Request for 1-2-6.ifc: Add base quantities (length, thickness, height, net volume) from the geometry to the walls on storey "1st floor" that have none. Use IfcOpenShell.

First a look at what the model holds.

```python
import ifcopenshell
import ifcopenshell.util.element
import ifcopenshell.util.unit

model = ifcopenshell.open("1-2-6.ifc")
print(model.schema)
for unit_type in ("LENGTHUNIT", "AREAUNIT", "VOLUMEUNIT"):
    print(unit_type, ifcopenshell.util.unit.calculate_unit_scale(model, unit_type))
storey = next(s for s in model.by_type("IfcBuildingStorey") if s.Name == "1st floor")
walls = [e for e in ifcopenshell.util.element.get_decomposition(storey) if e.is_a("IfcWall")]
for e in sorted(walls, key=lambda e: e.id()):
    print(e.id(), e.is_a(), e.Name, list(ifcopenshell.util.element.get_psets(e, qtos_only=True)), sep=" | ")
```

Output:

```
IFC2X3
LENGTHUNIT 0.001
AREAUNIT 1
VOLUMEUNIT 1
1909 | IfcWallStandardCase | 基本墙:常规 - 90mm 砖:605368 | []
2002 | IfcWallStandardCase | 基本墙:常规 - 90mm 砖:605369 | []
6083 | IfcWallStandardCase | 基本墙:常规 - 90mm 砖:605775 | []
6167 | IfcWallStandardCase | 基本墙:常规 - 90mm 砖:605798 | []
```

```python
import ifcopenshell
import ifcopenshell.api.pset
import ifcopenshell.geom
import ifcopenshell.util.element
import ifcopenshell.util.shape
import ifcopenshell.util.unit

model = ifcopenshell.open("1-2-6.ifc")
unit_scale = ifcopenshell.util.unit.calculate_unit_scale(model)
volume_scale = ifcopenshell.util.unit.calculate_unit_scale(model, "VOLUMEUNIT")
settings = ifcopenshell.geom.settings()

storey = next(s for s in model.by_type("IfcBuildingStorey") if s.Name == "1st floor")
walls = [e for e in ifcopenshell.util.element.get_decomposition(storey) if e.is_a("IfcWall")]

for e in sorted(walls, key=lambda e: e.id()):
    if ifcopenshell.util.element.get_psets(e, qtos_only=True, should_inherit=False):
        continue
    # Geometry comes back in metres, in the element's own axes.
    shape = ifcopenshell.geom.create_shape(settings, e)
    values = {
        "Length": ifcopenshell.util.shape.get_x(shape.geometry) / unit_scale,
        "Width": ifcopenshell.util.shape.get_y(shape.geometry) / unit_scale,
        "Height": ifcopenshell.util.shape.get_z(shape.geometry) / unit_scale,
        "NetVolume": ifcopenshell.util.shape.get_volume(shape.geometry) / volume_scale,
    }
    qto = ifcopenshell.api.pset.add_qto(model, product=e, name="BaseQuantities")
    ifcopenshell.api.pset.edit_qto(model, qto=qto, properties=values)
    print(e.id(), {k: round(v, 3) for k, v in values.items()})

model.write("1-2-6_updated.ifc")
```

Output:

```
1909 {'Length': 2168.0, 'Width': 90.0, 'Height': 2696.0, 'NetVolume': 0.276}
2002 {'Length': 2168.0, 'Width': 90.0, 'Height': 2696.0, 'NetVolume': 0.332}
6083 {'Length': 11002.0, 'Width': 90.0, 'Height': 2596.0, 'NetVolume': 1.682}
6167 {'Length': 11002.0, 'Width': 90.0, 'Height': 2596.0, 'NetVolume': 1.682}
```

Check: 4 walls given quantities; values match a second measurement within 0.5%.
